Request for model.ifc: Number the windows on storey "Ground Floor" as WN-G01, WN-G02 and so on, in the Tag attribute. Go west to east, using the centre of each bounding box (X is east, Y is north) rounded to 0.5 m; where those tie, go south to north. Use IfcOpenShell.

First a look at what the model holds.

```python
import ifcopenshell
import ifcopenshell.util.element
import ifcopenshell.util.placement

model = ifcopenshell.open("model.ifc")
print(model.schema)
storey = next(s for s in model.by_type("IfcBuildingStorey") if s.Name == "Ground Floor")
windows = [e for e in ifcopenshell.util.element.get_decomposition(storey) if e.is_a("IfcWindow")]
for e in sorted(windows, key=lambda e: e.id()):
    origin = ifcopenshell.util.placement.get_local_placement(e.ObjectPlacement)[:3, 3]
    print(e.id(), e.Tag, e.Name, origin.round(2) + 0.0, sep=" | ")
```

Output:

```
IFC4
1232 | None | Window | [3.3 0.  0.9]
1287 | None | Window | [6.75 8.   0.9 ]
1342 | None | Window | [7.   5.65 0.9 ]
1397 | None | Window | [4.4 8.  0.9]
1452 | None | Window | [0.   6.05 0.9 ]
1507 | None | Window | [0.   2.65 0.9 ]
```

```python
import ifcopenshell
import ifcopenshell.geom
import ifcopenshell.util.element
import ifcopenshell.util.shape

model = ifcopenshell.open("model.ifc")
settings = ifcopenshell.geom.settings()
settings.set("use-world-coords", True)


def centre(element):
    shape = ifcopenshell.geom.create_shape(settings, element)
    return ifcopenshell.util.shape.get_bbox_centroid(shape.geometry)


storey = next(s for s in model.by_type("IfcBuildingStorey") if s.Name == "Ground Floor")
windows = [e for e in ifcopenshell.util.element.get_decomposition(storey) if e.is_a("IfcWindow")]

# Insertion points can sit at a corner or the storey origin, so sort by the geometry (in metres).
centres = {e: centre(e) for e in windows}
windows.sort(key=lambda e: (round(centres[e][0] / 0.5), centres[e][1]))

for i, e in enumerate(windows, start=1):
    number = f"WN-G{i:02d}"
    e.Tag = number
    print(e.id(), number)

model.write("model_edited.ifc")
```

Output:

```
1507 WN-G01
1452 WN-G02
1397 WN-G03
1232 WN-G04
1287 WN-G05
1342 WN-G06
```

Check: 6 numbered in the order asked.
